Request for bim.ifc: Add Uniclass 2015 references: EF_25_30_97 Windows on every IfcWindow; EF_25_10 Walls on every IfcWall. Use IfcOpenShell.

First a look at what the model holds.

```python
import ifcopenshell

model = ifcopenshell.open("bim.ifc")
print(model.schema)
print("classifications:", [c.Name for c in model.by_type("IfcClassification")])
for ifc_class in ("IfcDoor", "IfcRoof", "IfcStair", "IfcWall", "IfcWindow"):
    print(ifc_class, len(model.by_type(ifc_class)))
```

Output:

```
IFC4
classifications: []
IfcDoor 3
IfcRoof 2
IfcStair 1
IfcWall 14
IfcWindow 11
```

```python
import ifcopenshell
import ifcopenshell.api.classification

model = ifcopenshell.open("bim.ifc")

system = ifcopenshell.api.classification.add_classification(model, classification="Uniclass 2015")

codes = {
    "IfcWindow": ("EF_25_30_97", "Windows"),
    "IfcWall": ("EF_25_10", "Walls"),
}
for ifc_class, (code, name) in codes.items():
    products = model.by_type(ifc_class)
    ifcopenshell.api.classification.add_reference(
        model, products=products, classification=system, identification=code, name=name
    )
    print(code, len(products))

model.write("bim_updated.ifc")
```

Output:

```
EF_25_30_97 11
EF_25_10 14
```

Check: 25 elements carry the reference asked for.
